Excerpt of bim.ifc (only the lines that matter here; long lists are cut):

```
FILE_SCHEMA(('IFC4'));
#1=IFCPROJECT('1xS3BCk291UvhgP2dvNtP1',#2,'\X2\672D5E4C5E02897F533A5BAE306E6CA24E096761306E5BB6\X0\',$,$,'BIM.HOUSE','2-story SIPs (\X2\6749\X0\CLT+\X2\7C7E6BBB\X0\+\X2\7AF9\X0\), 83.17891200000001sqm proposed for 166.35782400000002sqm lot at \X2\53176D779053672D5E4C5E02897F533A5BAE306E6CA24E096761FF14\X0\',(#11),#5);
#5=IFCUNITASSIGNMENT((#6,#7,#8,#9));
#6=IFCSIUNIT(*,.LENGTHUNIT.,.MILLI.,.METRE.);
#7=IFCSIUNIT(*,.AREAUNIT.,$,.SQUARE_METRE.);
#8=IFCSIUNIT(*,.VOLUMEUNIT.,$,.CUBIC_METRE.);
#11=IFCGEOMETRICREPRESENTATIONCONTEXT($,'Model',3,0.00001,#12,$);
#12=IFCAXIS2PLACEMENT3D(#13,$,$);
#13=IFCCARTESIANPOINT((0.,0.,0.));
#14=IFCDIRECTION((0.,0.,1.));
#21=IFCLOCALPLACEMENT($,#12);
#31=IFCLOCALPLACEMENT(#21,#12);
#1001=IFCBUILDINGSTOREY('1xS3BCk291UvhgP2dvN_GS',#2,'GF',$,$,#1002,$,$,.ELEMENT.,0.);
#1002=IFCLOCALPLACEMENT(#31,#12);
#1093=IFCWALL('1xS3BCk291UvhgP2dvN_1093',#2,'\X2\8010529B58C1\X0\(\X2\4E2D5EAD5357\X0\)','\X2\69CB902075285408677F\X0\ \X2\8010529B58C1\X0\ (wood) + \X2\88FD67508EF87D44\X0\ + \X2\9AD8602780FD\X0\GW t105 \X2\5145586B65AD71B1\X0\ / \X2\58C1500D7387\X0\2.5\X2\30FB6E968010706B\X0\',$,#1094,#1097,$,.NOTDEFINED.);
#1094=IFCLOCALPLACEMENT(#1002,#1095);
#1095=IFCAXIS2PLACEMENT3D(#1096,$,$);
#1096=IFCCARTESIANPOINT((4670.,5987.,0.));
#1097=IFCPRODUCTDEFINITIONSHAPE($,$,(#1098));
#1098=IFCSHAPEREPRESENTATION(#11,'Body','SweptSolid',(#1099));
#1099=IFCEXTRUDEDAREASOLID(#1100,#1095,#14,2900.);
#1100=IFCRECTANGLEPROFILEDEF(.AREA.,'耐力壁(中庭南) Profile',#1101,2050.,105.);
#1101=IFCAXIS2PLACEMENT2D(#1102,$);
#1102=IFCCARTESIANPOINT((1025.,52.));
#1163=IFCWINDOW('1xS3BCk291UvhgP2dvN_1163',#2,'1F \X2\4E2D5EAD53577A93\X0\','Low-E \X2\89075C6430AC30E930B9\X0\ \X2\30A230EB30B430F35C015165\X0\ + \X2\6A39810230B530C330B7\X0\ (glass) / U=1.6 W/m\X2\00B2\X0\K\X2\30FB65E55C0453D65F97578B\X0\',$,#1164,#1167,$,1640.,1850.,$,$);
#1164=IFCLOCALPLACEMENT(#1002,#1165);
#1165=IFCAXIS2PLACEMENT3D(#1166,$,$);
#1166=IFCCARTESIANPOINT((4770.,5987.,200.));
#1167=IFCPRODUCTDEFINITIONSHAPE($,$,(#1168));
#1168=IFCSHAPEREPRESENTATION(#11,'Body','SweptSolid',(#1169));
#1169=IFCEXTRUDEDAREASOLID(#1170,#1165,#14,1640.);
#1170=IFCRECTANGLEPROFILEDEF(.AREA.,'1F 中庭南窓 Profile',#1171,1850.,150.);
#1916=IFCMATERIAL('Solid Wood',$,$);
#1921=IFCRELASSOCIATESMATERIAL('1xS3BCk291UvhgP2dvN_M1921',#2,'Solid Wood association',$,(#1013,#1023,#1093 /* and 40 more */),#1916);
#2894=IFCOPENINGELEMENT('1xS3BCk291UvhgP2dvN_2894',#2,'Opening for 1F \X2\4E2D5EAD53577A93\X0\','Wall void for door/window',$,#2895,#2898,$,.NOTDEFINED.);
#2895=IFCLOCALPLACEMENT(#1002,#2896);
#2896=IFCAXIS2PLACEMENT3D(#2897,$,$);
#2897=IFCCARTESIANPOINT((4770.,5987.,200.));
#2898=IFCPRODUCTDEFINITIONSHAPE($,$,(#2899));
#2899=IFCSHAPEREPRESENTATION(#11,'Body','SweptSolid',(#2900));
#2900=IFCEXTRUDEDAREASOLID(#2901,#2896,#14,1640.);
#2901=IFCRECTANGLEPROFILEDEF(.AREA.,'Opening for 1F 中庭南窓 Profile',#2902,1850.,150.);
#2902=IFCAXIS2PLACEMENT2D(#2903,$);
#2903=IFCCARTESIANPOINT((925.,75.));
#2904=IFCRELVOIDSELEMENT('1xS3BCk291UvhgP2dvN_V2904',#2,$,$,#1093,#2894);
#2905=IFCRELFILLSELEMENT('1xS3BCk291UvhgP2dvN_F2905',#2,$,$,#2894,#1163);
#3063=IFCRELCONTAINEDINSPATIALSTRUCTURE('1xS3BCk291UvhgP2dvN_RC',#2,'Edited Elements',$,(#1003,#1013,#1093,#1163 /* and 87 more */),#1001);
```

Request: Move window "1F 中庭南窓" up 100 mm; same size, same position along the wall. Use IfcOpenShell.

```python
import numpy as np
import ifcopenshell
import ifcopenshell.api.geometry
import ifcopenshell.util.placement
import ifcopenshell.util.unit

model = ifcopenshell.open("bim.ifc")
unit_scale = ifcopenshell.util.unit.calculate_unit_scale(model)

window = model.by_id(1163)
opening = window.FillsVoids[0].RelatingOpeningElement
dz = 0.1 / unit_scale

shift = np.array([0.0, 0.0, dz])
# The window is not placed relative to its opening, so move both.
for product in (opening, window):
    matrix = ifcopenshell.util.placement.get_local_placement(product.ObjectPlacement)
    matrix[:3, 3] += shift
    ifcopenshell.api.geometry.edit_object_placement(model, product=product, matrix=matrix, is_si=False)

print(f"moved by {dz * unit_scale:+.3f} m")

model.write("bim_edited.ifc")
```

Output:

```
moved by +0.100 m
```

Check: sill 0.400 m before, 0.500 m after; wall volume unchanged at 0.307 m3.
